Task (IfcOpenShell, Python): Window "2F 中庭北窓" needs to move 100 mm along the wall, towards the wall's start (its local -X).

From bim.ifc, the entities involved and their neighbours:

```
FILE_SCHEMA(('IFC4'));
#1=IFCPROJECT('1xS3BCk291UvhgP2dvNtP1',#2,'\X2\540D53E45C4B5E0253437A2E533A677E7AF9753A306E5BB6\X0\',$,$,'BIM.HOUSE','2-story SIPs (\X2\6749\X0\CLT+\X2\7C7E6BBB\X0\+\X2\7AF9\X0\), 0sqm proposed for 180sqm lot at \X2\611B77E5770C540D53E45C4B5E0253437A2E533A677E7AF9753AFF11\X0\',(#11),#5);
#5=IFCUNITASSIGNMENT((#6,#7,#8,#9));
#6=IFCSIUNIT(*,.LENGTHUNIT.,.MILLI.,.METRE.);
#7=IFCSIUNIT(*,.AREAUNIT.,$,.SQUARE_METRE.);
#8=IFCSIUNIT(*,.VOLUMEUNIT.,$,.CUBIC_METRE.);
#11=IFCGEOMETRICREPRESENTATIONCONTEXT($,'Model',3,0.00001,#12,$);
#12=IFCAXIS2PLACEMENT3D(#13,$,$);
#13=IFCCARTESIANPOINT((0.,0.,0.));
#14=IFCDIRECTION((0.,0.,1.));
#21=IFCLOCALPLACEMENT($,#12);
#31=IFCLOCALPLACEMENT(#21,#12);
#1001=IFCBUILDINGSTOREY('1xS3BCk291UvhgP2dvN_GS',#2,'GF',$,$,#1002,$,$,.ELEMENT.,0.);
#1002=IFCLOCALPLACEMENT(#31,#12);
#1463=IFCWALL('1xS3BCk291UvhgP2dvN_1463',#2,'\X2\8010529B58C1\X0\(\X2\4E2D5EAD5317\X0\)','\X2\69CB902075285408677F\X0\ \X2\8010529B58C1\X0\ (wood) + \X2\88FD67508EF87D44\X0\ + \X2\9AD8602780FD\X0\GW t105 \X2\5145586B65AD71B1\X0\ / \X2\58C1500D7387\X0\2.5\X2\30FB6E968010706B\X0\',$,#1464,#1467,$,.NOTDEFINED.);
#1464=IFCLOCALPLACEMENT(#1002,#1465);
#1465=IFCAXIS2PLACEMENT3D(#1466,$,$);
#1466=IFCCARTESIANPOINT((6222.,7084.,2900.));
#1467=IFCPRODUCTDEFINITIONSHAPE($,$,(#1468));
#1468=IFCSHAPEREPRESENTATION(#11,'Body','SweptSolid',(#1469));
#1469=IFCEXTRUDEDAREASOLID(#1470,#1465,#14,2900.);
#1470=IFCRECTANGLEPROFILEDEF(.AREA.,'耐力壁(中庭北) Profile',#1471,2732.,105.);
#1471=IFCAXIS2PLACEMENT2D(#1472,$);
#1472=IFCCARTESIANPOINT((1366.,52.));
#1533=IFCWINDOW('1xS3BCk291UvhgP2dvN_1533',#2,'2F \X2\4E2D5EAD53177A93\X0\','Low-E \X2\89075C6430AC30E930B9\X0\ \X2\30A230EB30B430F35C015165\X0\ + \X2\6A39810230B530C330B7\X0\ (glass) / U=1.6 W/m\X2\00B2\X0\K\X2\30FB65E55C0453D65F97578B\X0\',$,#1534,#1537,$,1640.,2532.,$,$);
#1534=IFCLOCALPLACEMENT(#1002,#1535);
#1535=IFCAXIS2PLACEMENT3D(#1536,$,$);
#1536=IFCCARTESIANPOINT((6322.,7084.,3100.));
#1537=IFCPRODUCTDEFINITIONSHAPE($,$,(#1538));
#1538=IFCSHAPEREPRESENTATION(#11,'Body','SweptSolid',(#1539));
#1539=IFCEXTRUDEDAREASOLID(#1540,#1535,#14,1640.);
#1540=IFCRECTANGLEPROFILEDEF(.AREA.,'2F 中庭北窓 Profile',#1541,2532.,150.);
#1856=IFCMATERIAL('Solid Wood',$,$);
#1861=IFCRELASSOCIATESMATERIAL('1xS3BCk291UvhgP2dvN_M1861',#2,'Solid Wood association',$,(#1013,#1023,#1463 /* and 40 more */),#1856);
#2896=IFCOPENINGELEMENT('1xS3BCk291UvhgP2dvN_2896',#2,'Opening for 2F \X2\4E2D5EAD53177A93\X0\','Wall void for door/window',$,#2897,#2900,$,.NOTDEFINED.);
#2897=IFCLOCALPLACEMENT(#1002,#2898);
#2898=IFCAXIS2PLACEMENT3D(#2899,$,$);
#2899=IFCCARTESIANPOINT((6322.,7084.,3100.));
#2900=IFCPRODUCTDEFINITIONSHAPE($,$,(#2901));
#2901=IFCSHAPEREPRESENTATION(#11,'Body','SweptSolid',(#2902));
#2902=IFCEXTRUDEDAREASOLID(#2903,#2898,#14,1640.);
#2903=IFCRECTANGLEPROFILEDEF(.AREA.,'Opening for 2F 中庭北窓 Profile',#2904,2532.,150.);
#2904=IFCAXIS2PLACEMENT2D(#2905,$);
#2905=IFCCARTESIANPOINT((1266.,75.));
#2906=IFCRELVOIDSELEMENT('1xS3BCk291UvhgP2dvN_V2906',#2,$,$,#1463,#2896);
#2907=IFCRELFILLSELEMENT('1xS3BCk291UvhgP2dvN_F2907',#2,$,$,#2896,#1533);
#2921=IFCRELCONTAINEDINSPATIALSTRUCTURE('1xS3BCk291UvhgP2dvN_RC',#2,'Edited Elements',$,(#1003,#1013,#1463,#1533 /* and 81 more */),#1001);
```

```python
import ifcopenshell
import ifcopenshell.api.geometry
import ifcopenshell.util.placement
import ifcopenshell.util.unit

model = ifcopenshell.open("bim.ifc")
unit_scale = ifcopenshell.util.unit.calculate_unit_scale(model)

window = model.by_id(1533)
opening = window.FillsVoids[0].RelatingOpeningElement
wall = opening.VoidsElements[0].RelatingBuildingElement

wall_matrix = ifcopenshell.util.placement.get_local_placement(wall.ObjectPlacement)
shift = wall_matrix[:3, 0] * -0.1 / unit_scale
before = ifcopenshell.util.placement.get_local_placement(window.ObjectPlacement)[:3, 3].copy()

# The window is not placed relative to its opening, so move both.
for product in (opening, window):
    matrix = ifcopenshell.util.placement.get_local_placement(product.ObjectPlacement)
    matrix[:3, 3] += shift
    ifcopenshell.api.geometry.edit_object_placement(model, product=product, matrix=matrix, is_si=False)

after = ifcopenshell.util.placement.get_local_placement(window.ObjectPlacement)[:3, 3]
print("window moved by", (after - before).round(3) + 0.0)

model.write("bim_updated.ifc")
```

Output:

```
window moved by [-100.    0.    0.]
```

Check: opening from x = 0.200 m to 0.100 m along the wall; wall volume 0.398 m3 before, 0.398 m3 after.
